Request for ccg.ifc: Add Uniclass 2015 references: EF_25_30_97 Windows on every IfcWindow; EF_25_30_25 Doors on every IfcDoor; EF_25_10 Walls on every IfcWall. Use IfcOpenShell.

First a look at what the model holds.

```python
import ifcopenshell

model = ifcopenshell.open("ccg.ifc")
print(model.schema)
print("classifications:", [c.Name for c in model.by_type("IfcClassification")])
for ifc_class in ("IfcDoor", "IfcRoof", "IfcStair", "IfcWall", "IfcWindow"):
    print(ifc_class, len(model.by_type(ifc_class)))
```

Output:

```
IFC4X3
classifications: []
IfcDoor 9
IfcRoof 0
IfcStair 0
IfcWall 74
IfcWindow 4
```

```python
import ifcopenshell
import ifcopenshell.api.classification

model = ifcopenshell.open("ccg.ifc")

system = ifcopenshell.api.classification.add_classification(model, classification="Uniclass 2015")

codes = {
    "IfcWindow": ("EF_25_30_97", "Windows"),
    "IfcDoor": ("EF_25_30_25", "Doors"),
    "IfcWall": ("EF_25_10", "Walls"),
}
for ifc_class, (code, name) in codes.items():
    products = model.by_type(ifc_class)
    ifcopenshell.api.classification.add_reference(
        model, products=products, classification=system, identification=code, name=name
    )
    print(code, len(products))

model.write("ccg_updated.ifc")
```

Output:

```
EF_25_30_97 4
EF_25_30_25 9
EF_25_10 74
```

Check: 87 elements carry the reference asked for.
